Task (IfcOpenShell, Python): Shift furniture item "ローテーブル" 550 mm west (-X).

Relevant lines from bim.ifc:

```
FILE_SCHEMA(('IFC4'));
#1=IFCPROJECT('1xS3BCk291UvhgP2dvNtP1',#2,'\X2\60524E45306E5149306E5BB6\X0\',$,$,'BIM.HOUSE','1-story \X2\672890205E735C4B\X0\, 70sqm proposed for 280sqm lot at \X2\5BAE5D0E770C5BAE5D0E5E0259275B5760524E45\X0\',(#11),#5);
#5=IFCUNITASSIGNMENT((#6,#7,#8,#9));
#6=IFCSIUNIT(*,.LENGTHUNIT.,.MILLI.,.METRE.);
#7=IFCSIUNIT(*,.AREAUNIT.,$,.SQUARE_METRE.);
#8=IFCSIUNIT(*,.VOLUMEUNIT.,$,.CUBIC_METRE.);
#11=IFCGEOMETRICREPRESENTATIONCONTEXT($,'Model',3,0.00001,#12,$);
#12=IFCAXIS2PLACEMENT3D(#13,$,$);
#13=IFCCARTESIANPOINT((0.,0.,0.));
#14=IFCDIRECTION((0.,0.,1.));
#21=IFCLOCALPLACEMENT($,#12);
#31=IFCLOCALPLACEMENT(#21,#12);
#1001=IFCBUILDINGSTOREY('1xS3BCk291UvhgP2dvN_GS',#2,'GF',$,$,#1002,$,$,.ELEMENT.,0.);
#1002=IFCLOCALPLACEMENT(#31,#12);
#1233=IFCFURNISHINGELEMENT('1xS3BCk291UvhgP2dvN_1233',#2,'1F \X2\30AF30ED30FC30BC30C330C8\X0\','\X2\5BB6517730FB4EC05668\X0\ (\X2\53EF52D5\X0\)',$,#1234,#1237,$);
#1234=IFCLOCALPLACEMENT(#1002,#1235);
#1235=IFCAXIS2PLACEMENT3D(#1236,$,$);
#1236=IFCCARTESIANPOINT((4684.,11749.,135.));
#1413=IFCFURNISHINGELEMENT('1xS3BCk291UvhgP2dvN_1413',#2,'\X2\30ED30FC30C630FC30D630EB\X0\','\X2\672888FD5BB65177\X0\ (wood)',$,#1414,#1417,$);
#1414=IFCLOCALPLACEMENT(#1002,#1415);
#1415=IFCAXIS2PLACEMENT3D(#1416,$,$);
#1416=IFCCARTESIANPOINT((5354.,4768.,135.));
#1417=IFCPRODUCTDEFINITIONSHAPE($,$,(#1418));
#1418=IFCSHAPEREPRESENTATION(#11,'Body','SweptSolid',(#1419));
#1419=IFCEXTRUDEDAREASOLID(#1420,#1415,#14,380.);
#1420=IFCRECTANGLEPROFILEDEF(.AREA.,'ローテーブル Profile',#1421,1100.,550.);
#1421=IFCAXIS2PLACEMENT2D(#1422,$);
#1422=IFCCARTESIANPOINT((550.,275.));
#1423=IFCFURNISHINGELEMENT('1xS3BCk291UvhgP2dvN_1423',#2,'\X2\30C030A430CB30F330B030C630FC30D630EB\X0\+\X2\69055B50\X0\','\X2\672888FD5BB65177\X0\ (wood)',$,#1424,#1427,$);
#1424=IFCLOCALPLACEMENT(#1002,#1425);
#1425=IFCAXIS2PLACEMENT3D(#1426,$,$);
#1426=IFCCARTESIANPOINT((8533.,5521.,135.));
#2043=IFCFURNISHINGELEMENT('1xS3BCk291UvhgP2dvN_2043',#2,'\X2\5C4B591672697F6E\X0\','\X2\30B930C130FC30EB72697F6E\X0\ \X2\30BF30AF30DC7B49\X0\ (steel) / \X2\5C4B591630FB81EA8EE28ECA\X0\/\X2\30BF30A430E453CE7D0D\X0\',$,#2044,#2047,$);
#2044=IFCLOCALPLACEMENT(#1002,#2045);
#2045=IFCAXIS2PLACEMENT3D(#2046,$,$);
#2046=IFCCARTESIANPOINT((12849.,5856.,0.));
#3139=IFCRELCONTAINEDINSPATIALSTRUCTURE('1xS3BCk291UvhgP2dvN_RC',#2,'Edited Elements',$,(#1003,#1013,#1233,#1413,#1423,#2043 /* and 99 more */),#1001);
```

```python
import ifcopenshell
import ifcopenshell.api.geometry
import ifcopenshell.util.placement
import ifcopenshell.util.unit

model = ifcopenshell.open("bim.ifc")
unit_scale = ifcopenshell.util.unit.calculate_unit_scale(model)

item = model.by_guid("1xS3BCk291UvhgP2dvN_1413")
matrix = ifcopenshell.util.placement.get_local_placement(item.ObjectPlacement)
matrix[0, 3] -= 0.55 / unit_scale
ifcopenshell.api.geometry.edit_object_placement(model, product=item, matrix=matrix, is_si=False)

print(ifcopenshell.util.placement.get_local_placement(item.ObjectPlacement).round(3) + 0.0)

model.write("bim_edited.ifc")
```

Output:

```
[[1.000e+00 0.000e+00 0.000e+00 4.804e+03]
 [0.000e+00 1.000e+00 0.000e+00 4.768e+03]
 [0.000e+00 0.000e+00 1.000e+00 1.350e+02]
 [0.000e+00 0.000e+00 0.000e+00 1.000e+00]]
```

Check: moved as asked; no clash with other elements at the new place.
